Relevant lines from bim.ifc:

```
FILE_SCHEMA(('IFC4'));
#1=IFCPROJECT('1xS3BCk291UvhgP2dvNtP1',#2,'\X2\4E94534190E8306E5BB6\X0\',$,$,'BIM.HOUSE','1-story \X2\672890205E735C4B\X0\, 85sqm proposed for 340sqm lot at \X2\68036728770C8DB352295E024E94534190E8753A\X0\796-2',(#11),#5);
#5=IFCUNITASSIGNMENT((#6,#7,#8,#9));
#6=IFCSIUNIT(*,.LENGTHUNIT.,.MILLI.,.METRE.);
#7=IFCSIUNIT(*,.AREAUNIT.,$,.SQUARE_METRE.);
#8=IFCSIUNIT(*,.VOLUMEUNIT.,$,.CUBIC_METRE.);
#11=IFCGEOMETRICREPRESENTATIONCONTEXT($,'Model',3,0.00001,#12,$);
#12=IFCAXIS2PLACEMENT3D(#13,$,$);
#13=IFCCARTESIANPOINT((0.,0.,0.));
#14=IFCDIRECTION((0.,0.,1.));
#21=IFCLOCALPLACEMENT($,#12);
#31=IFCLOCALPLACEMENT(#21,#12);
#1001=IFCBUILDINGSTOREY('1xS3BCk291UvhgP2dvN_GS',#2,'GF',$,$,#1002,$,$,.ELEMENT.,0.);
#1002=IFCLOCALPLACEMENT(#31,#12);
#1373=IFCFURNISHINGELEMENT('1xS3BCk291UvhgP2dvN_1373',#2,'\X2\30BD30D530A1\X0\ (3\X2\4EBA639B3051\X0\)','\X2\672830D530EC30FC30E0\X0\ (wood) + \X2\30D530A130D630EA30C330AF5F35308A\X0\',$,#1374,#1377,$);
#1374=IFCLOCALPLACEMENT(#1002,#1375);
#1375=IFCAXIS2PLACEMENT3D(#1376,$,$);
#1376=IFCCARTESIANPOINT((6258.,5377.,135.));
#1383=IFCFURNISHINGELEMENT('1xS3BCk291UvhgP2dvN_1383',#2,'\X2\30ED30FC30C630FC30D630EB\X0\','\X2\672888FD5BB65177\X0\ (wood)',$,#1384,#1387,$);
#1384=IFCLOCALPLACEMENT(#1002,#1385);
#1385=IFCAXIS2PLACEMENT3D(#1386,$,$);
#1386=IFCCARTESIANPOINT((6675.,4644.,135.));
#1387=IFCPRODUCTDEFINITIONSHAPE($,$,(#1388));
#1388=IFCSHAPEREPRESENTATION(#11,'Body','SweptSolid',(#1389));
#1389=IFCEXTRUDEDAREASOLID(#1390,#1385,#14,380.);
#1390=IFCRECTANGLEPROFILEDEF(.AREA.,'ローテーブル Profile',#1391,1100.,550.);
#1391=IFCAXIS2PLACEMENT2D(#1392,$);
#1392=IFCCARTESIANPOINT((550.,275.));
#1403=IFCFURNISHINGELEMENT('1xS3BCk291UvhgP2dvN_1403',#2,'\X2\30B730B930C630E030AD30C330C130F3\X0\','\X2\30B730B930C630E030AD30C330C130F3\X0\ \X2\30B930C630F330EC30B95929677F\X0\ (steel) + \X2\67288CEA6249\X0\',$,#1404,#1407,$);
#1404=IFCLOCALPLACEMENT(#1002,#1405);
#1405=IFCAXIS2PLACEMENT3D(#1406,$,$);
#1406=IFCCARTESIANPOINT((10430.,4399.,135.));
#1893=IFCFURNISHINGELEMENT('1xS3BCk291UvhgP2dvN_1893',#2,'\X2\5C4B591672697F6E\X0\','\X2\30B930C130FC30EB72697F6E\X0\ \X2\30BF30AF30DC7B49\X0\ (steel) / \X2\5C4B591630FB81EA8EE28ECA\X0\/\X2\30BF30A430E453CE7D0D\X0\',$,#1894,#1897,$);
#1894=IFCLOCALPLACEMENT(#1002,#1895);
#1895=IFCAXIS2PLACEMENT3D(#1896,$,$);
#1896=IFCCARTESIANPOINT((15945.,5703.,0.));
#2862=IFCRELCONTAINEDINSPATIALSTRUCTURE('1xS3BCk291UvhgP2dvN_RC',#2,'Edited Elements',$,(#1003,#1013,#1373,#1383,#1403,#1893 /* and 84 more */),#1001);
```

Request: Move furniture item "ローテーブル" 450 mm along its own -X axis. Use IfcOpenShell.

```python
import ifcopenshell
import ifcopenshell.api.geometry
import ifcopenshell.util.placement

model = ifcopenshell.open("bim.ifc")

item = model.by_guid("1xS3BCk291UvhgP2dvN_1383")
matrix = ifcopenshell.util.placement.get_local_placement(item.ObjectPlacement)
matrix[:3, 3] -= matrix[:3, 0] * 450.0
ifcopenshell.api.geometry.edit_object_placement(model, product=item, matrix=matrix, is_si=False)

print(ifcopenshell.util.placement.get_local_placement(item.ObjectPlacement).round(3) + 0.0)

model.write("bim_v2.ifc")
```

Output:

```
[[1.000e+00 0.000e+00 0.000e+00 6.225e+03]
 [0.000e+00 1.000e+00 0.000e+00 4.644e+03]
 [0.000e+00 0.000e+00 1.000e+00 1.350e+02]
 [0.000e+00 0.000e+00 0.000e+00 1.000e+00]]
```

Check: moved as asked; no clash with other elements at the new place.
